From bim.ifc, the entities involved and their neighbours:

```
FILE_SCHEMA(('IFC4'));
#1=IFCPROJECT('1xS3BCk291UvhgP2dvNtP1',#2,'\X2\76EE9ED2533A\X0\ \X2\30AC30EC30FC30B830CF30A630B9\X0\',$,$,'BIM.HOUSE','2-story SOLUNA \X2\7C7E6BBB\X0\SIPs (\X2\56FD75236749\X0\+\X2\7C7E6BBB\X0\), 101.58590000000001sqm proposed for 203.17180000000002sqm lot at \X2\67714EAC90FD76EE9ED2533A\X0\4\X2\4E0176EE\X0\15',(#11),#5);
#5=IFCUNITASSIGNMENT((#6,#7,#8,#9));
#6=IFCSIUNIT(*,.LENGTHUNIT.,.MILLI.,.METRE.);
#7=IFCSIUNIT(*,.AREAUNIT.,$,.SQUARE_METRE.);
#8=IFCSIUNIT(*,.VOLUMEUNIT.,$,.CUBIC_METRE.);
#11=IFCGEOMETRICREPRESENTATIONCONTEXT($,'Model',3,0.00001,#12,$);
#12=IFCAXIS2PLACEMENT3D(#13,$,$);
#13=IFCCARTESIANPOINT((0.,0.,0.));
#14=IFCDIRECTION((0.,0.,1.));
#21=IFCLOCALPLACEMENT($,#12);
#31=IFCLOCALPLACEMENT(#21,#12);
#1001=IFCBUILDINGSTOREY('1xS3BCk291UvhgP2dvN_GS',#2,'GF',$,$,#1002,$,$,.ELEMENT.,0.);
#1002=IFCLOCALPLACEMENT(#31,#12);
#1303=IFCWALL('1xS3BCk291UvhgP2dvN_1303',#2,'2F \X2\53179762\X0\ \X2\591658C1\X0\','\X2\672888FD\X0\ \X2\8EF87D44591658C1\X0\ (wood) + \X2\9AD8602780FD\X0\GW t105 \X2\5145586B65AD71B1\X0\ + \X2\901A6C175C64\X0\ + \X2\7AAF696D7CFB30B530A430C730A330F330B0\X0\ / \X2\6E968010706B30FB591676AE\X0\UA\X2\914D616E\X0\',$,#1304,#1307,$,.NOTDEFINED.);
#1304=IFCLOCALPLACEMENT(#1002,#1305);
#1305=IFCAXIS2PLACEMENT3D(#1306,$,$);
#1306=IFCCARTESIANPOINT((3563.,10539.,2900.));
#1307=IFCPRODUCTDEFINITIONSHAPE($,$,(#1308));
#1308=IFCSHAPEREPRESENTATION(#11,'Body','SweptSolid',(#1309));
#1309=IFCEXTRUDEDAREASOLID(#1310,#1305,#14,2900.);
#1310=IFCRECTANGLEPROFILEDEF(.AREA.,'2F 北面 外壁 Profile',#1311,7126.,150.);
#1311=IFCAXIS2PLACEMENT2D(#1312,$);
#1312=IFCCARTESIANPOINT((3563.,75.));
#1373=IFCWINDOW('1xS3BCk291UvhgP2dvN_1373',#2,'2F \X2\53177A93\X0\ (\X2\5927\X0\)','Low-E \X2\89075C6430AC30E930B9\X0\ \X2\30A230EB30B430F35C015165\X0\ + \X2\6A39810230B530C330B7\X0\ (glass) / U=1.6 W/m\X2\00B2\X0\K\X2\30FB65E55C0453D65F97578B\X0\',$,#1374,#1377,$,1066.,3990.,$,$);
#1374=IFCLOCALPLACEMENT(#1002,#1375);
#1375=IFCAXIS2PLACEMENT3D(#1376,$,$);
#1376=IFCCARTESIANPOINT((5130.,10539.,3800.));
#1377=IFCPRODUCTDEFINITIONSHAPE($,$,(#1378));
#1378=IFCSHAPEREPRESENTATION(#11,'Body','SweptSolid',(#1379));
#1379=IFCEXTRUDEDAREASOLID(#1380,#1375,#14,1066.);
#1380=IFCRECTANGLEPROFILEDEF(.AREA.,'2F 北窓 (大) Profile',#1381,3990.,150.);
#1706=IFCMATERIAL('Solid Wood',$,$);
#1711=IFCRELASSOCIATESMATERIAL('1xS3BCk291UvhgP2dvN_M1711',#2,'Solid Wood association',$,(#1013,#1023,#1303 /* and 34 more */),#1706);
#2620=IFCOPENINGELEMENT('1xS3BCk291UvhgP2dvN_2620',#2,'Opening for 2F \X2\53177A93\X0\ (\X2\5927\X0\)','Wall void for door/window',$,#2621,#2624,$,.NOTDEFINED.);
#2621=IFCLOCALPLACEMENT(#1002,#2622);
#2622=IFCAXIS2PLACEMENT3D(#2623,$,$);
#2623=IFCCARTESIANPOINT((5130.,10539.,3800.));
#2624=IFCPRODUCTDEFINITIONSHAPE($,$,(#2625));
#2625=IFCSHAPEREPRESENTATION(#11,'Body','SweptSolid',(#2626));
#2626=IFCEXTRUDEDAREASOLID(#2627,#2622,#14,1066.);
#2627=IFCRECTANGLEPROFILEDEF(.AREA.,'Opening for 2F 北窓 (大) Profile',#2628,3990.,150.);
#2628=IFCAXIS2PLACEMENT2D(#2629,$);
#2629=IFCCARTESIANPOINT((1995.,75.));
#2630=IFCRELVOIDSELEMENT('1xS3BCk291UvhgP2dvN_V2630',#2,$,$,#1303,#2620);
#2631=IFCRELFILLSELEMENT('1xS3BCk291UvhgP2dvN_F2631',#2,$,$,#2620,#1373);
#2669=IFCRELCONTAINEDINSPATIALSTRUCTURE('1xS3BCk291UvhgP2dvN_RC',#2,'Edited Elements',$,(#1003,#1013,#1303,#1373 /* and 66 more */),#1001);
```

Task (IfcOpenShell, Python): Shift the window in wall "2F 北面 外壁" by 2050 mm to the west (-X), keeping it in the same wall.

```python
import ifcopenshell
import ifcopenshell.api.geometry
import ifcopenshell.util.placement
import ifcopenshell.util.unit

model = ifcopenshell.open("bim.ifc")
unit_scale = ifcopenshell.util.unit.calculate_unit_scale(model)

window = model.by_guid("1xS3BCk291UvhgP2dvN_1373")
opening = window.FillsVoids[0].RelatingOpeningElement
wall = opening.VoidsElements[0].RelatingBuildingElement

wall_matrix = ifcopenshell.util.placement.get_local_placement(wall.ObjectPlacement)
shift = wall_matrix[:3, 0] * -2.05 / unit_scale
before = ifcopenshell.util.placement.get_local_placement(window.ObjectPlacement)[:3, 3].copy()

# The window is not placed relative to its opening, so move both.
for product in (opening, window):
    matrix = ifcopenshell.util.placement.get_local_placement(product.ObjectPlacement)
    matrix[:3, 3] += shift
    ifcopenshell.api.geometry.edit_object_placement(model, product=product, matrix=matrix, is_si=False)

after = ifcopenshell.util.placement.get_local_placement(window.ObjectPlacement)[:3, 3]
print("window moved by", (after - before).round(3) + 0.0)

model.write("bim_v2.ifc")
```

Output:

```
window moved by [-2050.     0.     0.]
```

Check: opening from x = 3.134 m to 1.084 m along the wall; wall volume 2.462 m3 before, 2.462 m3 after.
